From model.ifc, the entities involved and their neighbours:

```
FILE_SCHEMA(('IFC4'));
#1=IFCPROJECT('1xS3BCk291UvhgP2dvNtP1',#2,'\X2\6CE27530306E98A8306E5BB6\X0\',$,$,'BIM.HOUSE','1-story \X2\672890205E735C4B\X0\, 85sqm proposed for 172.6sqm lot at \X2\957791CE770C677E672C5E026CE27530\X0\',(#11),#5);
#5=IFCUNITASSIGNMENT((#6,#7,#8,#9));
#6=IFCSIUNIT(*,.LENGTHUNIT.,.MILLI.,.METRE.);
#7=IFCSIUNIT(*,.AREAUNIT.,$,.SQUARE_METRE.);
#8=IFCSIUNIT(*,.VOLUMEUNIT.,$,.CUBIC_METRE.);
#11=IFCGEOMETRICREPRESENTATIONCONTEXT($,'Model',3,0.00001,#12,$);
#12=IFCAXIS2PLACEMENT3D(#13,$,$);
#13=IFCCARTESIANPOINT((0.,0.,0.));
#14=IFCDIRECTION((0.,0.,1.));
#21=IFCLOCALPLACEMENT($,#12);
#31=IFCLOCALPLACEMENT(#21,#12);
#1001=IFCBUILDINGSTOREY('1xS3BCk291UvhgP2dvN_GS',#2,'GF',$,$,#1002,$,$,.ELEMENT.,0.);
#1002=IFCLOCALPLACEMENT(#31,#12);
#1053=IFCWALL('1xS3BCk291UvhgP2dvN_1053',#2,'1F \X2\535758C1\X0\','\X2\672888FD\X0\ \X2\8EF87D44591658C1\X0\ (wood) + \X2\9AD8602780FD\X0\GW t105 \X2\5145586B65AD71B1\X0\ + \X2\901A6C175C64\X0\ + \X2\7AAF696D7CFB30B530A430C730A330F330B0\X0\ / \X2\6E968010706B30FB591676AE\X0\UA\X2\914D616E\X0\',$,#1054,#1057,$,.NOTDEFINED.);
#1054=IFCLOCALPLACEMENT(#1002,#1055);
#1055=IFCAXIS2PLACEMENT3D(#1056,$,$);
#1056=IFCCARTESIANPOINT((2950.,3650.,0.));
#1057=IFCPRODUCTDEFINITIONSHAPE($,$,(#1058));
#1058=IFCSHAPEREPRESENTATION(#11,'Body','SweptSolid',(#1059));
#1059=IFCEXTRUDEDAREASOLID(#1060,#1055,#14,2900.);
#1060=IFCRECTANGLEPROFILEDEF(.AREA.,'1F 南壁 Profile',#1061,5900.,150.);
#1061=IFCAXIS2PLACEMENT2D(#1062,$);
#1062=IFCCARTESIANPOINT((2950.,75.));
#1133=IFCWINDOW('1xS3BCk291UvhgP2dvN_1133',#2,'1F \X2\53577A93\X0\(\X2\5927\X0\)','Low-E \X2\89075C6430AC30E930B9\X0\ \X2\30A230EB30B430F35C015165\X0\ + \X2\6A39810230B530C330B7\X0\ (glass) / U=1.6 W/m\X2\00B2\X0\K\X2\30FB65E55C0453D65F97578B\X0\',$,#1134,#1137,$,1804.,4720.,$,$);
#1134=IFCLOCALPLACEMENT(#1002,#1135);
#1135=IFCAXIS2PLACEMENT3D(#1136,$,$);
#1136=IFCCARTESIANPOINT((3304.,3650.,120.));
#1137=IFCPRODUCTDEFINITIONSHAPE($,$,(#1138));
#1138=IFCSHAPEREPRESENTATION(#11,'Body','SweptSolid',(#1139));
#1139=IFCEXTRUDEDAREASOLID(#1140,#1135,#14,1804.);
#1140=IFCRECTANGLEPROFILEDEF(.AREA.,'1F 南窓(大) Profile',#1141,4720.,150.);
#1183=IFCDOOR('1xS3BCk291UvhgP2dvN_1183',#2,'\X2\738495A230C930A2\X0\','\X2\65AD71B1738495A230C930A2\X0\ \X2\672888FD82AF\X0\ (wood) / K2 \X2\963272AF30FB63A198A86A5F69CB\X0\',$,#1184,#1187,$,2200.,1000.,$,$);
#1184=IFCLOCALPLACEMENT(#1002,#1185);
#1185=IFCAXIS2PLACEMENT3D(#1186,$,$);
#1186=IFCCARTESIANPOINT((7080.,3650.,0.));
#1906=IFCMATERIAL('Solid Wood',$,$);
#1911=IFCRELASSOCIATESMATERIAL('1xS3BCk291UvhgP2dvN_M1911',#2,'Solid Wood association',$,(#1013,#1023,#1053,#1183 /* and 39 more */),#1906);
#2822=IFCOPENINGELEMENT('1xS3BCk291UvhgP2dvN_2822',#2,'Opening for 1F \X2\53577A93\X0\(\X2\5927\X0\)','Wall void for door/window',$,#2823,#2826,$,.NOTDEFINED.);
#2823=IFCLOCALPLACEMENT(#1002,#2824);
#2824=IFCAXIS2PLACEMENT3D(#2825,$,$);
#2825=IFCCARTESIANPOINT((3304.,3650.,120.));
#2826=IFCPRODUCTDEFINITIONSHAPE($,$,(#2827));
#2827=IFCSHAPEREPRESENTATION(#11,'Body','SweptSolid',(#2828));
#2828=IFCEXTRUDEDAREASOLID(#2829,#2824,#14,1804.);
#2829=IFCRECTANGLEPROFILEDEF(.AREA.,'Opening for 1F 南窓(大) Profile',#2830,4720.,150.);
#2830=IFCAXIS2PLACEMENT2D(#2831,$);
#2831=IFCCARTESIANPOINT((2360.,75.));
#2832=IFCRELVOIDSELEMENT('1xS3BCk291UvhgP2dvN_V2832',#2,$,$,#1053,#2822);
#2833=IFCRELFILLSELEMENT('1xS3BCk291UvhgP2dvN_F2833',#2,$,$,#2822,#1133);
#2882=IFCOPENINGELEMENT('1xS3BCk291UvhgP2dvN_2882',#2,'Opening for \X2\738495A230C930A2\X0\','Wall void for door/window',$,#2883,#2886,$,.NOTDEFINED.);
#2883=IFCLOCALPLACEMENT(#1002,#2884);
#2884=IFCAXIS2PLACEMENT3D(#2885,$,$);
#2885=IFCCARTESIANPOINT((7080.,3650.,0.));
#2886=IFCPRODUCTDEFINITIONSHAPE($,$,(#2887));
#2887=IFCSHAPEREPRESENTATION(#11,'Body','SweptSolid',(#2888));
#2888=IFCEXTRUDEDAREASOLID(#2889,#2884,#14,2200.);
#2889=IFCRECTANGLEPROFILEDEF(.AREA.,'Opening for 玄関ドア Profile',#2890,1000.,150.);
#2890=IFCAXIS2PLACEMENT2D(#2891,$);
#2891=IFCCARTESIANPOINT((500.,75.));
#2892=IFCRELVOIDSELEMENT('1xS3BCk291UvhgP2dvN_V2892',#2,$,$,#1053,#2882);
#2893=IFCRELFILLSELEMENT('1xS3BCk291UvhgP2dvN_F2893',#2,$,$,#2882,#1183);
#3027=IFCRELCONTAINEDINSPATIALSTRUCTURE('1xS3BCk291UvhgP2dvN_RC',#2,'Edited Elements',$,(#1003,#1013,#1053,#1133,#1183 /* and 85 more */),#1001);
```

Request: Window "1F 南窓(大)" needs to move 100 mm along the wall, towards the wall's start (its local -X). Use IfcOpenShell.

```python
import ifcopenshell
import ifcopenshell.api.geometry
import ifcopenshell.util.placement

model = ifcopenshell.open("model.ifc")

window = model.by_guid("1xS3BCk291UvhgP2dvN_1133")
opening = window.FillsVoids[0].RelatingOpeningElement
wall = opening.VoidsElements[0].RelatingBuildingElement

wall_matrix = ifcopenshell.util.placement.get_local_placement(wall.ObjectPlacement)
shift = wall_matrix[:3, 0] * -100.0
before = ifcopenshell.util.placement.get_local_placement(window.ObjectPlacement)[:3, 3].copy()

# The window is not placed relative to its opening, so move both.
for product in (opening, window):
    matrix = ifcopenshell.util.placement.get_local_placement(product.ObjectPlacement)
    matrix[:3, 3] += shift
    ifcopenshell.api.geometry.edit_object_placement(model, product=product, matrix=matrix, is_si=False)

after = ifcopenshell.util.placement.get_local_placement(window.ObjectPlacement)[:3, 3]
print("window moved by", (after - before).round(3) + 0.0)

model.write("model_v2.ifc")
```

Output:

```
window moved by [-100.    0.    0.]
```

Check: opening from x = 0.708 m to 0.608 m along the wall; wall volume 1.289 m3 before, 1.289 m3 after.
